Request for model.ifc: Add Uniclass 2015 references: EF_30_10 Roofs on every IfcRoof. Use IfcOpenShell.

First a look at what the model holds.

```python
import ifcopenshell

model = ifcopenshell.open("model.ifc")
print(model.schema)
print("classifications:", [c.Name for c in model.by_type("IfcClassification")])
for ifc_class in ("IfcDoor", "IfcRoof", "IfcStair", "IfcWall", "IfcWindow"):
    print(ifc_class, len(model.by_type(ifc_class)))
```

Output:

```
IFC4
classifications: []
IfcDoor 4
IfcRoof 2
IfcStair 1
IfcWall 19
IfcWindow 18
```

```python
import ifcopenshell
import ifcopenshell.api.classification

model = ifcopenshell.open("model.ifc")

system = ifcopenshell.api.classification.add_classification(model, classification="Uniclass 2015")

codes = {
    "IfcRoof": ("EF_30_10", "Roofs"),
}
for ifc_class, (code, name) in codes.items():
    products = model.by_type(ifc_class)
    ifcopenshell.api.classification.add_reference(
        model, products=products, classification=system, identification=code, name=name
    )
    print(code, len(products))

model.write("model_rev.ifc")
```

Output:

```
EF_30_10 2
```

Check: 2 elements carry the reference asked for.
